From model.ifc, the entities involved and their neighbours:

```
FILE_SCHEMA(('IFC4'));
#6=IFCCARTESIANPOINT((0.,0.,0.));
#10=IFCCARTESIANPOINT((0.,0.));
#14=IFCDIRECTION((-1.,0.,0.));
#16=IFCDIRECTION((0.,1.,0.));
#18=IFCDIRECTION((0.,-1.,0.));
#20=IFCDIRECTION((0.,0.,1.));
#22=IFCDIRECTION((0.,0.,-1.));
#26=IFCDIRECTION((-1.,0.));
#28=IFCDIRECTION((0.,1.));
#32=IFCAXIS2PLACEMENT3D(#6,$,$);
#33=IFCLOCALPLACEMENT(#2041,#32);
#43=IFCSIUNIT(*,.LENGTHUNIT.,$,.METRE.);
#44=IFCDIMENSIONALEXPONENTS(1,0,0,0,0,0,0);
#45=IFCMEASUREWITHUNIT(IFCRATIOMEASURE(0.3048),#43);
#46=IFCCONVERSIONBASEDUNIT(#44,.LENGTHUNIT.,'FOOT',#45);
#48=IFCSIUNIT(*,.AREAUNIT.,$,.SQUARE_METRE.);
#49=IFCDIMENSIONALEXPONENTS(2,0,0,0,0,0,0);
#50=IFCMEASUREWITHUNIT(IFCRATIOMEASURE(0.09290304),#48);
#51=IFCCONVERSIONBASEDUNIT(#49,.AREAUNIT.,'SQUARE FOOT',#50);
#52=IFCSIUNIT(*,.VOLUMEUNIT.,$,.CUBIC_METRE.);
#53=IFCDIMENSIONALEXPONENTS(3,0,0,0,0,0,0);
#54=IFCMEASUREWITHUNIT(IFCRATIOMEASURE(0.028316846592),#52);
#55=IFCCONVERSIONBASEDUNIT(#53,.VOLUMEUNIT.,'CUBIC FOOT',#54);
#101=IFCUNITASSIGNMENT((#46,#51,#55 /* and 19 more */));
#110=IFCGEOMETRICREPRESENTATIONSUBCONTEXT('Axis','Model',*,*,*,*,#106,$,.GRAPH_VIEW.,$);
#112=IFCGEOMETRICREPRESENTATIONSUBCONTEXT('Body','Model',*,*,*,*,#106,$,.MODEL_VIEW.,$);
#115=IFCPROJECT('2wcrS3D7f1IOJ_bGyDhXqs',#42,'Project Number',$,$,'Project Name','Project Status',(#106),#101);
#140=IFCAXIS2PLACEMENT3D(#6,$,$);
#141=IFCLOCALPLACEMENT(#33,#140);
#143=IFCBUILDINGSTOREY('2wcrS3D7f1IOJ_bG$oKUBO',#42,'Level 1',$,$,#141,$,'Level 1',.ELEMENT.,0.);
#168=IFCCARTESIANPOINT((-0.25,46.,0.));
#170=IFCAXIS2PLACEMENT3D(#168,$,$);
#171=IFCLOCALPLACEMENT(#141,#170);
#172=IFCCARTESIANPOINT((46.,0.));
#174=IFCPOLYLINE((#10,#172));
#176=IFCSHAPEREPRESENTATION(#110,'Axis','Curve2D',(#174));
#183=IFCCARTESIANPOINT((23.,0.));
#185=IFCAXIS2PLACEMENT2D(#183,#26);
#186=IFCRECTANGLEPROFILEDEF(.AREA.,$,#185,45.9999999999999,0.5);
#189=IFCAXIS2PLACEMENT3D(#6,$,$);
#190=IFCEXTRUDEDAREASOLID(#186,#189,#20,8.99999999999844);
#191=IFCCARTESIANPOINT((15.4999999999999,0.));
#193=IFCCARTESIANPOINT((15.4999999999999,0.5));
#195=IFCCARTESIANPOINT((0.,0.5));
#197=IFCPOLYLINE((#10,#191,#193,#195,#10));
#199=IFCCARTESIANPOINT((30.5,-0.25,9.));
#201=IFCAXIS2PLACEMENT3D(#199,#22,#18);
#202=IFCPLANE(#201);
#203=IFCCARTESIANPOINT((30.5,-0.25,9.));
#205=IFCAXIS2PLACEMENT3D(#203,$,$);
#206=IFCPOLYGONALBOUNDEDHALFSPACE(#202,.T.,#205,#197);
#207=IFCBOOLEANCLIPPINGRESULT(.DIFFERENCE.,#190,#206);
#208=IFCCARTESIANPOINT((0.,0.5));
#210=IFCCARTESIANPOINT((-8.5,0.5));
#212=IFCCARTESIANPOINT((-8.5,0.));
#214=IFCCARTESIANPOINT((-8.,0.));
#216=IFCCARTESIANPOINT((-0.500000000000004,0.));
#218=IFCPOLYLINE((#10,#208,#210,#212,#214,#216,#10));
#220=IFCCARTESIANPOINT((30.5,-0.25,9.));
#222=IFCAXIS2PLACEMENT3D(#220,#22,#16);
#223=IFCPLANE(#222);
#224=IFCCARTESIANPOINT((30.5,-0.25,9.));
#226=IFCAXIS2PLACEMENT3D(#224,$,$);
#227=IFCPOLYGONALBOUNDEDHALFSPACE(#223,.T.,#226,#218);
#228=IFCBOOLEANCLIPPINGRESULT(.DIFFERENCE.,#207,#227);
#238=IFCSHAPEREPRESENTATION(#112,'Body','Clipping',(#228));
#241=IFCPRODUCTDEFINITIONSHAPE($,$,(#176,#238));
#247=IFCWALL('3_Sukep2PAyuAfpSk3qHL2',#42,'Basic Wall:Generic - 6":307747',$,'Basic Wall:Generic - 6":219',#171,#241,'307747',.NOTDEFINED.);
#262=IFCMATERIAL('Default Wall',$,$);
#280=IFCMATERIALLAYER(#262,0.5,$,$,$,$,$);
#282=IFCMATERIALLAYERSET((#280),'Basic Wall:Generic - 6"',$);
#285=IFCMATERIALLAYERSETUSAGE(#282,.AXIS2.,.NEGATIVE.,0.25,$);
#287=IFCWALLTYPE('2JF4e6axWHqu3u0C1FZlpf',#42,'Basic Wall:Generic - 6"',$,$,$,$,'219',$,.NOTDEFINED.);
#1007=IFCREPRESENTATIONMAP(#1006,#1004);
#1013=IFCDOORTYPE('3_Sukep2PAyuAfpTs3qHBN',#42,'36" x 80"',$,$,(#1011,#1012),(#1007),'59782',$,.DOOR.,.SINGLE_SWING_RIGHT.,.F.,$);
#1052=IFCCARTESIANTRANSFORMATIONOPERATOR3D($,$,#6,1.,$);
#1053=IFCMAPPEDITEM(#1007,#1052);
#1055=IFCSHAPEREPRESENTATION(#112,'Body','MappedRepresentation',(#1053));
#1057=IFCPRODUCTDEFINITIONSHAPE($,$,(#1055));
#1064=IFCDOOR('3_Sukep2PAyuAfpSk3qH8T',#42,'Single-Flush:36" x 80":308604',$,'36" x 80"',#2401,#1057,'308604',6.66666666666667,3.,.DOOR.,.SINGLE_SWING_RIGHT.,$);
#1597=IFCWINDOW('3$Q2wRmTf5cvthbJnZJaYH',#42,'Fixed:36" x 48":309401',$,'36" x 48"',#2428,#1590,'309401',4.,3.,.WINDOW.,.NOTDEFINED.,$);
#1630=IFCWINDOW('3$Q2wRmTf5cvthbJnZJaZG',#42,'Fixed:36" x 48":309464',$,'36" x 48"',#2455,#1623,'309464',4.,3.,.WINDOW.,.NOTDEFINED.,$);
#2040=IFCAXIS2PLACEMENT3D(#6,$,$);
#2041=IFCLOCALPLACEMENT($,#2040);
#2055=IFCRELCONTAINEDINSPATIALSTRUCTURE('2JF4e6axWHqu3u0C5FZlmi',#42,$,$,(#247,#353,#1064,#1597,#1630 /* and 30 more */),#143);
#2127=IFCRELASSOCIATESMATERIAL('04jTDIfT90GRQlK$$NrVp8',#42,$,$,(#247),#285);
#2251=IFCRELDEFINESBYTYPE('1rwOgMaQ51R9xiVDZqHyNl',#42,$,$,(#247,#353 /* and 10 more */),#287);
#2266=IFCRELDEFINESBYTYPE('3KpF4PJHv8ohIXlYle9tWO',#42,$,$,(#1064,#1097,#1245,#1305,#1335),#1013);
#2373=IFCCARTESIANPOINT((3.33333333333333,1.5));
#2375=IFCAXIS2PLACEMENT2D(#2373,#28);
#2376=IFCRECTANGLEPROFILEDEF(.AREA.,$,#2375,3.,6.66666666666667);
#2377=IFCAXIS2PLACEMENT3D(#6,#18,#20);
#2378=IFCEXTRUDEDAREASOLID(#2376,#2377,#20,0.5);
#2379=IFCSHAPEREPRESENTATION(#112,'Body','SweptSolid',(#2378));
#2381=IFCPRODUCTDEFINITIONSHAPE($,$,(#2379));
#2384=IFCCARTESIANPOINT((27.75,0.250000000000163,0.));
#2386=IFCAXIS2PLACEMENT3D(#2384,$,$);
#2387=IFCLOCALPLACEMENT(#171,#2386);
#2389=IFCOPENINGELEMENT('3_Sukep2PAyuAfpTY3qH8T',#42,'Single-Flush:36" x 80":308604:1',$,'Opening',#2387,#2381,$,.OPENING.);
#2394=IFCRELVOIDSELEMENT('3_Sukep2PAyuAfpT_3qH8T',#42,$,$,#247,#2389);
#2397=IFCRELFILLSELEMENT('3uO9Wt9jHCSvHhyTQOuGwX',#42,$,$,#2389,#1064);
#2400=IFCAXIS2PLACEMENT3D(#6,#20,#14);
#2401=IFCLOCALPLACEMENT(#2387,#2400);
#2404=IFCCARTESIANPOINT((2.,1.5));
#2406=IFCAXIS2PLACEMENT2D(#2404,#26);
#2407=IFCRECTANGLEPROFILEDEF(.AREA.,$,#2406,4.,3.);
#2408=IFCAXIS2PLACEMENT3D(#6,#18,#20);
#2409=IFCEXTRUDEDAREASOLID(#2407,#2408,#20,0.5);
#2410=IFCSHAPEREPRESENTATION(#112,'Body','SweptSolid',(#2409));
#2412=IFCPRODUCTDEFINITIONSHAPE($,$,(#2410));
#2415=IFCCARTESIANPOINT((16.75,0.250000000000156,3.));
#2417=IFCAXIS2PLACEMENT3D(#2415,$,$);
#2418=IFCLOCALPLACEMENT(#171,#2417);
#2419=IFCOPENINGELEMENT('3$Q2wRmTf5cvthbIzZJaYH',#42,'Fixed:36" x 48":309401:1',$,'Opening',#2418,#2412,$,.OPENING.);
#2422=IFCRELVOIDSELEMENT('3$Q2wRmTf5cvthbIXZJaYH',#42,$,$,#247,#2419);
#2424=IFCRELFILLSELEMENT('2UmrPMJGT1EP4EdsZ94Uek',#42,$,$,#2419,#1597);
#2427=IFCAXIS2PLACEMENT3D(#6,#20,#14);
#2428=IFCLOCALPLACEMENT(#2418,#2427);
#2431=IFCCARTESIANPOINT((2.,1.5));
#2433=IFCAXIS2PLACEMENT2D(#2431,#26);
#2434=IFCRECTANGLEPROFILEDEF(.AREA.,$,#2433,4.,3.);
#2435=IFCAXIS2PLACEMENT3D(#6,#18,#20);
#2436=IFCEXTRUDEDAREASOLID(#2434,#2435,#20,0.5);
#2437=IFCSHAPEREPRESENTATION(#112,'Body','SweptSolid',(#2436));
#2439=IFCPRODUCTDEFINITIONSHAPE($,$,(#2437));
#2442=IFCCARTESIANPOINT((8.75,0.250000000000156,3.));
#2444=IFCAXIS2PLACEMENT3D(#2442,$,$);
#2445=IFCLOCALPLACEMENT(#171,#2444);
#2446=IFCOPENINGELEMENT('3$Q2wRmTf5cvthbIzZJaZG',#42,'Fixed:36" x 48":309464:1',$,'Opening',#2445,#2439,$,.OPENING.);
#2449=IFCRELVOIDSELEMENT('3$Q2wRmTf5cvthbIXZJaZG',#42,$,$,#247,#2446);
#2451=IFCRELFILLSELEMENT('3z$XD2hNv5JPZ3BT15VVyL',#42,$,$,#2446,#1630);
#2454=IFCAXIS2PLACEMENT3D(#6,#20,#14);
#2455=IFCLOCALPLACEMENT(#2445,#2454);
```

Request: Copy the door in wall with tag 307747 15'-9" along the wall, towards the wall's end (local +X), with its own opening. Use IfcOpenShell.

```python
import ifcopenshell
import ifcopenshell.api.feature
import ifcopenshell.api.geometry
import ifcopenshell.api.root
import ifcopenshell.geom
import ifcopenshell.util.element
import ifcopenshell.util.placement
import ifcopenshell.util.shape
import ifcopenshell.util.unit

model = ifcopenshell.open("model.ifc")
unit_scale = ifcopenshell.util.unit.calculate_unit_scale(model)
settings = ifcopenshell.geom.settings()


def volume(element):
    """Net volume in cubic metres, openings subtracted."""
    shape = ifcopenshell.geom.create_shape(settings, element)
    return ifcopenshell.util.shape.get_volume(shape.geometry)


def reuse_history(source, copy):
    """copy_class also copies each property set's owner history, people and application; keep the originals."""
    for rel in copy.IsDefinedBy:
        if rel.is_a("IfcRelDefinesByProperties") and (history := rel.RelatingPropertyDefinition.OwnerHistory):
            rel.RelatingPropertyDefinition.OwnerHistory = source.OwnerHistory
            ifcopenshell.util.element.remove_deep2(model, history)


door = model.by_guid("3_Sukep2PAyuAfpSk3qH8T")
opening = door.FillsVoids[0].RelatingOpeningElement
wall = opening.VoidsElements[0].RelatingBuildingElement
before = volume(wall)
shift = ifcopenshell.util.placement.get_local_placement(wall.ObjectPlacement)[:3, 0] * 189 * 0.0254 / unit_scale

# copy_class copies the void relationship, type, container and properties, but no geometry.
new_opening = ifcopenshell.api.root.copy_class(model, product=opening)
new_opening.Representation = ifcopenshell.util.element.copy_deep(
    model, opening.Representation, exclude=["IfcGeometricRepresentationContext", "IfcRepresentationMap"]
)
new_opening.Name = 'Single-Flush:36" x 80"'
new_door = ifcopenshell.api.root.copy_class(model, product=door)
new_door.Representation = ifcopenshell.util.element.copy_deep(
    model, door.Representation, exclude=["IfcGeometricRepresentationContext", "IfcRepresentationMap"]
)
new_door.Name = 'Single-Flush:36" x 80"'
new_door.Tag = None
reuse_history(door, new_door)
ifcopenshell.api.feature.add_filling(model, opening=new_opening, element=new_door)

for old, new in ((opening, new_opening), (door, new_door)):
    matrix = ifcopenshell.util.placement.get_local_placement(old.ObjectPlacement)
    matrix[:3, 3] += shift
    ifcopenshell.api.geometry.edit_object_placement(model, product=new, matrix=matrix, is_si=False)

after = volume(wall)

print(f"wall volume {before:.3f} -> {after:.3f} m3")

model.write("model_edited.ifc")
```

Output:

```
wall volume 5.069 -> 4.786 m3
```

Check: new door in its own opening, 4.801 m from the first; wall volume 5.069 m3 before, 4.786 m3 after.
